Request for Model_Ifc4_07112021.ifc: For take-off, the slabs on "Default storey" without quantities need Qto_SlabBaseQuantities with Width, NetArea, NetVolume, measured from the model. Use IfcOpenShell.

First a look at what the model holds.

```python
import ifcopenshell
import ifcopenshell.util.element
import ifcopenshell.util.unit

model = ifcopenshell.open("Model_Ifc4_07112021.ifc")
print(model.schema)
for unit_type in ("LENGTHUNIT", "AREAUNIT", "VOLUMEUNIT"):
    print(unit_type, ifcopenshell.util.unit.calculate_unit_scale(model, unit_type))
storey = next(s for s in model.by_type("IfcBuildingStorey") if s.Name == "Default storey")
slabs = [e for e in ifcopenshell.util.element.get_decomposition(storey) if e.is_a("IfcSlab")]
for e in sorted(slabs, key=lambda e: e.id()):
    print(e.id(), e.is_a(), e.Name, list(ifcopenshell.util.element.get_psets(e, qtos_only=True)), sep=" | ")
```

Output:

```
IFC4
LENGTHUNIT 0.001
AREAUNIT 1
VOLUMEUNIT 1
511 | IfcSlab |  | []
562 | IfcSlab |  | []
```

```python
import ifcopenshell
import ifcopenshell.api.pset
import ifcopenshell.geom
import ifcopenshell.util.element
import ifcopenshell.util.shape
import ifcopenshell.util.unit

model = ifcopenshell.open("Model_Ifc4_07112021.ifc")
unit_scale = ifcopenshell.util.unit.calculate_unit_scale(model)
area_scale = ifcopenshell.util.unit.calculate_unit_scale(model, "AREAUNIT")
volume_scale = ifcopenshell.util.unit.calculate_unit_scale(model, "VOLUMEUNIT")
settings = ifcopenshell.geom.settings()

storey = next(s for s in model.by_type("IfcBuildingStorey") if s.Name == "Default storey")
slabs = [e for e in ifcopenshell.util.element.get_decomposition(storey) if e.is_a("IfcSlab")]

for e in sorted(slabs, key=lambda e: e.id()):
    if ifcopenshell.util.element.get_psets(e, qtos_only=True, should_inherit=False):
        continue
    # Geometry comes back in metres, in the element's own axes.
    shape = ifcopenshell.geom.create_shape(settings, e)
    values = {
        "Width": ifcopenshell.util.shape.get_z(shape.geometry) / unit_scale,
        "NetArea": ifcopenshell.util.shape.get_footprint_area(shape.geometry) / area_scale,
        "NetVolume": ifcopenshell.util.shape.get_volume(shape.geometry) / volume_scale,
    }
    qto = ifcopenshell.api.pset.add_qto(model, product=e, name="Qto_SlabBaseQuantities")
    ifcopenshell.api.pset.edit_qto(model, qto=qto, properties=values)
    print(e.id(), {k: round(v, 3) for k, v in values.items()})

model.write("Model_Ifc4_07112021_v2.ifc")
```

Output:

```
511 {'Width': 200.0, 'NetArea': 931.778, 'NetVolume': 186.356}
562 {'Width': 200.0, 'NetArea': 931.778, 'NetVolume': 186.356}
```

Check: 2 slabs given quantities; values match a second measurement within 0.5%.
